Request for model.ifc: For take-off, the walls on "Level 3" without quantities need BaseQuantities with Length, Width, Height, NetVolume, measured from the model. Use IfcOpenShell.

First a look at what the model holds.

```python
import ifcopenshell
import ifcopenshell.util.element
import ifcopenshell.util.unit

model = ifcopenshell.open("model.ifc")
print(model.schema)
for unit_type in ("LENGTHUNIT", "AREAUNIT", "VOLUMEUNIT"):
    print(unit_type, ifcopenshell.util.unit.calculate_unit_scale(model, unit_type))
storey = next(s for s in model.by_type("IfcBuildingStorey") if s.Name == "Level 3")
walls = [e for e in ifcopenshell.util.element.get_decomposition(storey) if e.is_a("IfcWall")]
for e in sorted(walls, key=lambda e: e.id()):
    print(e.id(), e.is_a(), e.Name, list(ifcopenshell.util.element.get_psets(e, qtos_only=True)), sep=" | ")
```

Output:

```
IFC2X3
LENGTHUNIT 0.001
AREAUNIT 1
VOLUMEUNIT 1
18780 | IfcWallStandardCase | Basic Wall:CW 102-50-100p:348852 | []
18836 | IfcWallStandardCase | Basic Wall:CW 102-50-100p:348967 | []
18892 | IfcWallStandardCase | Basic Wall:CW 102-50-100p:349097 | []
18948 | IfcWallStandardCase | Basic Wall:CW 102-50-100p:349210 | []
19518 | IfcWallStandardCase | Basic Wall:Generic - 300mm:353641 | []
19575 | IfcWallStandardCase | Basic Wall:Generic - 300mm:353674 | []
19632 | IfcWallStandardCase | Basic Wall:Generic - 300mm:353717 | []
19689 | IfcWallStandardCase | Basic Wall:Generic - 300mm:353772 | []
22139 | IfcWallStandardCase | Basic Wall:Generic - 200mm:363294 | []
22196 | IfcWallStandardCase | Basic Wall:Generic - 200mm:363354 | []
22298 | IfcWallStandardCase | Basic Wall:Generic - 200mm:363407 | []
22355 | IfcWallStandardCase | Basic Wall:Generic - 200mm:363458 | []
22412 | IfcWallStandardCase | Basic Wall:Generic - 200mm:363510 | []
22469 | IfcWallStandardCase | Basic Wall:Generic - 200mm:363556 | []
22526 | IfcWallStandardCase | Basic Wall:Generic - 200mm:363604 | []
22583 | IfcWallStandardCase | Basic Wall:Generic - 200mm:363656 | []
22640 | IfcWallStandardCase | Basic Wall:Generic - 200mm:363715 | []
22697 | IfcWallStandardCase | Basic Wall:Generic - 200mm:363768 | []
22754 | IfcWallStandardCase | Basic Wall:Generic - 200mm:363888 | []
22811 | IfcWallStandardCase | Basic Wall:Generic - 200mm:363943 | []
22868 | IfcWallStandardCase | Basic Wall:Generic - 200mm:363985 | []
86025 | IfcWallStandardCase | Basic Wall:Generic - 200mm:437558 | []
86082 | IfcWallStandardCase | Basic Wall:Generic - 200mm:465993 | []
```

```python
import ifcopenshell
import ifcopenshell.api.pset
import ifcopenshell.geom
import ifcopenshell.util.element
import ifcopenshell.util.shape
import ifcopenshell.util.unit

model = ifcopenshell.open("model.ifc")
unit_scale = ifcopenshell.util.unit.calculate_unit_scale(model)
volume_scale = ifcopenshell.util.unit.calculate_unit_scale(model, "VOLUMEUNIT")
settings = ifcopenshell.geom.settings()

storey = next(s for s in model.by_type("IfcBuildingStorey") if s.Name == "Level 3")
walls = [e for e in ifcopenshell.util.element.get_decomposition(storey) if e.is_a("IfcWall")]

for e in sorted(walls, key=lambda e: e.id()):
    if ifcopenshell.util.element.get_psets(e, qtos_only=True, should_inherit=False):
        continue
    # Geometry comes back in metres, in the element's own axes.
    shape = ifcopenshell.geom.create_shape(settings, e)
    values = {
        "Length": ifcopenshell.util.shape.get_x(shape.geometry) / unit_scale,
        "Width": ifcopenshell.util.shape.get_y(shape.geometry) / unit_scale,
        "Height": ifcopenshell.util.shape.get_z(shape.geometry) / unit_scale,
        "NetVolume": ifcopenshell.util.shape.get_volume(shape.geometry) / volume_scale,
    }
    qto = ifcopenshell.api.pset.add_qto(model, product=e, name="BaseQuantities")
    ifcopenshell.api.pset.edit_qto(model, qto=qto, properties=values)
    print(e.id(), {k: round(v, 3) for k, v in values.items()})

model.write("model_updated.ifc")
```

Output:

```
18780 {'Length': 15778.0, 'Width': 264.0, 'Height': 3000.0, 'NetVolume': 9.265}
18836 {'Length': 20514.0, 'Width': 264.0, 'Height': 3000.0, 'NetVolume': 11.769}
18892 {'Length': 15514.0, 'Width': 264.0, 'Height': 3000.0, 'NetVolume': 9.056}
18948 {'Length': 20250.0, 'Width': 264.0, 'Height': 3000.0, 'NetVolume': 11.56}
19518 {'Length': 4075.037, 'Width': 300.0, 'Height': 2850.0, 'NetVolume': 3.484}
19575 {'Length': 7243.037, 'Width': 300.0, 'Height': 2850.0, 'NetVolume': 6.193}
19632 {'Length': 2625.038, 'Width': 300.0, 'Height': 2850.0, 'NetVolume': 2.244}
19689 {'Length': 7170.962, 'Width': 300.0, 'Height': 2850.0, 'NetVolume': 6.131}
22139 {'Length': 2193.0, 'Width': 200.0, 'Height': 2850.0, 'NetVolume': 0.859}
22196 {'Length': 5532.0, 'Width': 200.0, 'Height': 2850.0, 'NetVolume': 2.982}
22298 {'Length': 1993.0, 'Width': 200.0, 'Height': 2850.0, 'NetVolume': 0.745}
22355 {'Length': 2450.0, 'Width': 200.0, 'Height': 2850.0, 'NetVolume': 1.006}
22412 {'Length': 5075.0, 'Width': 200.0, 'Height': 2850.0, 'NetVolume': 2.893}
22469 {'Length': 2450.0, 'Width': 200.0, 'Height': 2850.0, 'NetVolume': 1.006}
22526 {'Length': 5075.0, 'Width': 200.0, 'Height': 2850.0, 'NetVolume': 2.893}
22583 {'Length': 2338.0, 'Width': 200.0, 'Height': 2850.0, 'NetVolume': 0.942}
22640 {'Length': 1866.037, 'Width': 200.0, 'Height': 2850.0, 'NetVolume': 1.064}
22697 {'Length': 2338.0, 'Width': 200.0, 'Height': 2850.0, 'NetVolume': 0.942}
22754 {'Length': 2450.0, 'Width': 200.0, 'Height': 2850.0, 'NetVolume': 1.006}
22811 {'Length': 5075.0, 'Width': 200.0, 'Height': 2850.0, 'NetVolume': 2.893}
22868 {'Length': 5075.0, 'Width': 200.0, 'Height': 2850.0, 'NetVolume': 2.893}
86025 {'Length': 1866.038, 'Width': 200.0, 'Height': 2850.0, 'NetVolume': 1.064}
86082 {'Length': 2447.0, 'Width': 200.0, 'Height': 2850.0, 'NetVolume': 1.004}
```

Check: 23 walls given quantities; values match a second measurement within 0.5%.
